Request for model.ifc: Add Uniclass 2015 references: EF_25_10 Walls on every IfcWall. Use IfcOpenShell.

First a look at what the model holds.

```python
import ifcopenshell

model = ifcopenshell.open("model.ifc")
print(model.schema)
print("classifications:", [c.Name for c in model.by_type("IfcClassification")])
for ifc_class in ("IfcDoor", "IfcRoof", "IfcStair", "IfcWall", "IfcWindow"):
    print(ifc_class, len(model.by_type(ifc_class)))
```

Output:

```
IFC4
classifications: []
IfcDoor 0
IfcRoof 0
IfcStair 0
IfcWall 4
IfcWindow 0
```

```python
import ifcopenshell
import ifcopenshell.api.classification

model = ifcopenshell.open("model.ifc")

system = ifcopenshell.api.classification.add_classification(model, classification="Uniclass 2015")

codes = {
    "IfcWall": ("EF_25_10", "Walls"),
}
for ifc_class, (code, name) in codes.items():
    products = model.by_type(ifc_class)
    ifcopenshell.api.classification.add_reference(
        model, products=products, classification=system, identification=code, name=name
    )
    print(code, len(products))

model.write("model_edited.ifc")
```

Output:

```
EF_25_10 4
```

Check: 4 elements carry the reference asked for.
